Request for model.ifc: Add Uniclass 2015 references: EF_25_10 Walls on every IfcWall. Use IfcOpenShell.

First a look at what the model holds.

```python
import ifcopenshell

model = ifcopenshell.open("model.ifc")
print(model.schema)
print("classifications:", [c.Name for c in model.by_type("IfcClassification")])
for ifc_class in ("IfcDoor", "IfcRoof", "IfcStair", "IfcWall", "IfcWindow"):
    print(ifc_class, len(model.by_type(ifc_class)))
```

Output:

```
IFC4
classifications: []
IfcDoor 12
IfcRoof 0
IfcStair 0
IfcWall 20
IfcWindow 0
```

```python
import ifcopenshell
import ifcopenshell.api.classification

model = ifcopenshell.open("model.ifc")

system = ifcopenshell.api.classification.add_classification(model, classification="Uniclass 2015")

codes = {
    "IfcWall": ("EF_25_10", "Walls"),
}
for ifc_class, (code, name) in codes.items():
    products = model.by_type(ifc_class)
    ifcopenshell.api.classification.add_reference(
        model, products=products, classification=system, identification=code, name=name
    )
    print(code, len(products))

model.write("model_rev.ifc")
```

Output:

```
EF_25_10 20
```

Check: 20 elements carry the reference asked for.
